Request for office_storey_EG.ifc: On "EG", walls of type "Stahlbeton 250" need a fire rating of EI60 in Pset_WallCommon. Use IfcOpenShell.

First a look at what the model holds.

```python
import ifcopenshell
import ifcopenshell.util.element

model = ifcopenshell.open("office_storey_EG.ifc")
print(model.schema)
storey = next(s for s in model.by_type("IfcBuildingStorey") if s.Name == "EG")
walls = [e for e in ifcopenshell.util.element.get_decomposition(storey) if e.is_a("IfcWall")]
seen = {}
for e in walls:
    element_type = ifcopenshell.util.element.get_type(e)
    key = (element_type.Name if element_type != e and element_type else None, ifcopenshell.util.element.get_pset(e, "Pset_WallCommon", "FireRating"))
    seen[key] = seen.get(key, 0) + 1
for (name, value), count in sorted(seen.items(), key=str):
    print(count, "x", name, "|", value)
```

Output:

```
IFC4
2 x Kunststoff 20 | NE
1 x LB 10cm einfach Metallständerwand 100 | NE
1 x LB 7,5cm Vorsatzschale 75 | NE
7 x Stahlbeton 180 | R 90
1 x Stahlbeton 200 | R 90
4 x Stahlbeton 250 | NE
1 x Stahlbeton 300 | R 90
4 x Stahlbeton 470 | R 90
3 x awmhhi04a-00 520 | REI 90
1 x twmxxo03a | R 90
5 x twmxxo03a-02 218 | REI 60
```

```python
import ifcopenshell
import ifcopenshell.api.pset
import ifcopenshell.util.element

model = ifcopenshell.open("office_storey_EG.ifc")

storey = next(s for s in model.by_type("IfcBuildingStorey") if s.Name == "EG")
walls = [e for e in ifcopenshell.util.element.get_decomposition(storey) if e.is_a("IfcWall")]

count = 0
for e in walls:
    element_type = ifcopenshell.util.element.get_type(e)
    if element_type in (None, e) or element_type.Name != "Stahlbeton 250":
        continue
    # add_pset returns the element's existing set when there is one.
    pset = ifcopenshell.api.pset.add_pset(model, product=e, name="Pset_WallCommon")
    ifcopenshell.api.pset.edit_pset(model, pset=pset, properties={"FireRating": "EI60"})
    count += 1

print(count, "walls updated")

model.write("office_storey_EG-out.ifc")
```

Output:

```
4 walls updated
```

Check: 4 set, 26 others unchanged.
